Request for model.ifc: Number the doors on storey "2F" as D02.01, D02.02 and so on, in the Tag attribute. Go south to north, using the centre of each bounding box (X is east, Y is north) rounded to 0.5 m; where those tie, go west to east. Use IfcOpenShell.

First a look at what the model holds.

```python
import ifcopenshell
import ifcopenshell.util.element
import ifcopenshell.util.placement

model = ifcopenshell.open("model.ifc")
print(model.schema)
storey = next(s for s in model.by_type("IfcBuildingStorey") if s.Name == "2F")
doors = [e for e in ifcopenshell.util.element.get_decomposition(storey) if e.is_a("IfcDoor")]
for e in sorted(doors, key=lambda e: e.id()):
    origin = ifcopenshell.util.placement.get_local_placement(e.ObjectPlacement)[:3, 3]
    print(e.id(), e.Tag, e.Name, origin.round(2) + 0.0, sep=" | ")
```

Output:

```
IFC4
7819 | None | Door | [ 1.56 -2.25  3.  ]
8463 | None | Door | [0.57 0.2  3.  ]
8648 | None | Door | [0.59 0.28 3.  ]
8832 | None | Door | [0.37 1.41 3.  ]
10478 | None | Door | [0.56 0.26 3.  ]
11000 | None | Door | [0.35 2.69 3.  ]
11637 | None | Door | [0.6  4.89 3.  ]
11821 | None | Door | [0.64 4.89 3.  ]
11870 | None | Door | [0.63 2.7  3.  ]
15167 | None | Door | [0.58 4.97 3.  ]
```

```python
import ifcopenshell
import ifcopenshell.geom
import ifcopenshell.util.element
import ifcopenshell.util.shape

model = ifcopenshell.open("model.ifc")
settings = ifcopenshell.geom.settings()
settings.set("use-world-coords", True)


def centre(element):
    shape = ifcopenshell.geom.create_shape(settings, element)
    return ifcopenshell.util.shape.get_bbox_centroid(shape.geometry)


storey = next(s for s in model.by_type("IfcBuildingStorey") if s.Name == "2F")
doors = [e for e in ifcopenshell.util.element.get_decomposition(storey) if e.is_a("IfcDoor")]

# Insertion points can sit at a corner or the storey origin, so sort by the geometry (in metres).
centres = {e: centre(e) for e in doors}
doors.sort(key=lambda e: (round(centres[e][1] / 0.5), centres[e][0]))

for i, e in enumerate(doors, start=1):
    number = f"D02.{i:02d}"
    e.Tag = number
    print(e.id(), number)

model.write("model-out.ifc")
```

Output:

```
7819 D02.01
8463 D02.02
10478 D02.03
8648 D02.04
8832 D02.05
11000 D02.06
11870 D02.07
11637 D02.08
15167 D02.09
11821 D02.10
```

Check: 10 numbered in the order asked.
